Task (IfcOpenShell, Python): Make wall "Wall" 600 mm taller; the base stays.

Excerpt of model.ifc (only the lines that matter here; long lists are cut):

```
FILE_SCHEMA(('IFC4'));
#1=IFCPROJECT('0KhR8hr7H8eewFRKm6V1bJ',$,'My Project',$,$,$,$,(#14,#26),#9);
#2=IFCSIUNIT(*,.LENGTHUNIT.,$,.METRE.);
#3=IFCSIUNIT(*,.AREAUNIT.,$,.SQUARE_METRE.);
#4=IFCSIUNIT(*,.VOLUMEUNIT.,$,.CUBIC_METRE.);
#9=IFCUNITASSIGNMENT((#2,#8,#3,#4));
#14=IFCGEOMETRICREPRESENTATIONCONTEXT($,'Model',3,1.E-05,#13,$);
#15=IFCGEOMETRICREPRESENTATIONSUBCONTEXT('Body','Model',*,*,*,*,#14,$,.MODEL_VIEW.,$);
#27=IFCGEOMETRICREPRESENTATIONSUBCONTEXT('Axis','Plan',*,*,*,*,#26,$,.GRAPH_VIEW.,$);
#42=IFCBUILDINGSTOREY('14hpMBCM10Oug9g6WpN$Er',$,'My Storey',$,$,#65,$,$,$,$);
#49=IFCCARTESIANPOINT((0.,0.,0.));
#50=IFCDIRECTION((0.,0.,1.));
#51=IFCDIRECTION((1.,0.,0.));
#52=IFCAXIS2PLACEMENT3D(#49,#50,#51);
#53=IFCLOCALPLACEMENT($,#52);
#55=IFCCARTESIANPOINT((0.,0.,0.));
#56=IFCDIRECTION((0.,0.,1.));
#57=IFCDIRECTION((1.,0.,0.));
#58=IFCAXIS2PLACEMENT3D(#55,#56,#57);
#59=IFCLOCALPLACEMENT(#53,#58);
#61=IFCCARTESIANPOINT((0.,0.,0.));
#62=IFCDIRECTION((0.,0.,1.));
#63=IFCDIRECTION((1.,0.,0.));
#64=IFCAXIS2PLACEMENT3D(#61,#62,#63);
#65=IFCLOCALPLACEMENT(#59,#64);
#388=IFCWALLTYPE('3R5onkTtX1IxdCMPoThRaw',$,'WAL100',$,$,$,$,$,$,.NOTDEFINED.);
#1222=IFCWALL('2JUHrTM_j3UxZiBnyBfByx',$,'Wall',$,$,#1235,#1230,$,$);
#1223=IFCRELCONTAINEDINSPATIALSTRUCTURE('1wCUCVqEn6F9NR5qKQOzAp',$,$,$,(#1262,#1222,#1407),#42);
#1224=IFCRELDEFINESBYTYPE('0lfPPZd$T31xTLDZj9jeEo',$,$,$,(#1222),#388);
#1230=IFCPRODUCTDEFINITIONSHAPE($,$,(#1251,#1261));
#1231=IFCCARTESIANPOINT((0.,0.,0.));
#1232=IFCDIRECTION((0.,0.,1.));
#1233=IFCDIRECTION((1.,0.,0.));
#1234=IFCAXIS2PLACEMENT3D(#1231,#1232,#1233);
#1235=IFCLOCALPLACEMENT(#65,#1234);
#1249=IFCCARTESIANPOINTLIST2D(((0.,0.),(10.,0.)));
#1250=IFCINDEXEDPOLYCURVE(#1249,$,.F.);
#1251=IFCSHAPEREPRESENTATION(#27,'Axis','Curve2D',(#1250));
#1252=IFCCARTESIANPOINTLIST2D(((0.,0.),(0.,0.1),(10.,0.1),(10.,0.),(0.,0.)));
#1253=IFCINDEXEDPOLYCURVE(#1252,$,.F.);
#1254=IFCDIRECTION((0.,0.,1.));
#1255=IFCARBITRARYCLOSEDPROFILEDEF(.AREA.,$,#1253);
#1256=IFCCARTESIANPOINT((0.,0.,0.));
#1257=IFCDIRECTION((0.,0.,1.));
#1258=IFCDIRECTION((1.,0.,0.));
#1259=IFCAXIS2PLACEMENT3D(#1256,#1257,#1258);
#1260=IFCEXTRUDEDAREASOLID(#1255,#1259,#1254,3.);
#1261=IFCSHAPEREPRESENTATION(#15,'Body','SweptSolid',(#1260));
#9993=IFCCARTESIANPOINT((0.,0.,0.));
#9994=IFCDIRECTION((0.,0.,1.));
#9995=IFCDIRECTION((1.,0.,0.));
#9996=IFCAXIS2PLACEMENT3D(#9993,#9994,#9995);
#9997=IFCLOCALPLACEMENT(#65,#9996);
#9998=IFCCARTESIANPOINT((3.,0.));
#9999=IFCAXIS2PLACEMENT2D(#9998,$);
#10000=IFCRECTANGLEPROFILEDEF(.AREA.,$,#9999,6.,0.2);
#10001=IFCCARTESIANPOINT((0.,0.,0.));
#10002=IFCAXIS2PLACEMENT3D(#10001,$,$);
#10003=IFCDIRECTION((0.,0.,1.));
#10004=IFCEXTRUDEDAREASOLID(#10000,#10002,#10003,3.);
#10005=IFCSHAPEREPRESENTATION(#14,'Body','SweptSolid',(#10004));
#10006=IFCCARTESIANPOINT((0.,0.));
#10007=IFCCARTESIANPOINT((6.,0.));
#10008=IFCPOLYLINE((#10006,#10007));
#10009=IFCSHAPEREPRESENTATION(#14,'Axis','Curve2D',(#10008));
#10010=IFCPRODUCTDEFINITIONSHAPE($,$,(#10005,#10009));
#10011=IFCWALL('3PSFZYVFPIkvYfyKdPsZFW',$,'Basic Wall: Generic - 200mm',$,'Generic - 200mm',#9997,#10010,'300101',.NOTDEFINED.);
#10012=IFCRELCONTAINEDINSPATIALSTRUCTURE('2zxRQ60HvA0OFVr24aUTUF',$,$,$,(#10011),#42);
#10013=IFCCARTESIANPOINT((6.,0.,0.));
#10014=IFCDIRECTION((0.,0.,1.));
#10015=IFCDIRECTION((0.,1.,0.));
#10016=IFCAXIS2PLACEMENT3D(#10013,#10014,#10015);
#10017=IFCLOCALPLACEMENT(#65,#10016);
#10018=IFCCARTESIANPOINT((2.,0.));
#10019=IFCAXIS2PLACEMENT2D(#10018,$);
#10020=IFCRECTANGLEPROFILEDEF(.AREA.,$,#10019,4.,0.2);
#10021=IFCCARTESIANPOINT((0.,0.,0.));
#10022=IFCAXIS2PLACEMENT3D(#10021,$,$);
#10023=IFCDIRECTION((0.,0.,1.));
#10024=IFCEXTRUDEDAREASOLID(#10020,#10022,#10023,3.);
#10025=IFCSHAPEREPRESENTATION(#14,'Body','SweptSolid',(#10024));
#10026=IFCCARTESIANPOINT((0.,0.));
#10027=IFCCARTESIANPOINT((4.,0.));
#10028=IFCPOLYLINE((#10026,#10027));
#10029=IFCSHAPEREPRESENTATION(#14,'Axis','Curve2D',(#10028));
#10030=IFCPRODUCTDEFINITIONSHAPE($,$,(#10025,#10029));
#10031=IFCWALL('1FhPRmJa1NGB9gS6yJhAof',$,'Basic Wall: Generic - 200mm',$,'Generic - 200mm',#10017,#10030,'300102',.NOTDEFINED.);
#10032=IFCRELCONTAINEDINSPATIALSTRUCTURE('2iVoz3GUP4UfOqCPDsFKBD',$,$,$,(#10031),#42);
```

```python
import ifcopenshell
import ifcopenshell.geom
import ifcopenshell.util.representation
import ifcopenshell.util.shape

model = ifcopenshell.open("model.ifc")
settings = ifcopenshell.geom.settings()


def volume(element):
    """Net volume in cubic metres, openings subtracted."""
    shape = ifcopenshell.geom.create_shape(settings, element)
    return ifcopenshell.util.shape.get_volume(shape.geometry)


wall = model.by_guid("2JUHrTM_j3UxZiBnyBfByx")
before = volume(wall)

body = ifcopenshell.util.representation.get_representation(wall, "Model", "Body")
solid = body.Items[0]
old_height = solid.Depth
solid.Depth += 0.6
after = volume(wall)

print(f"height {old_height:g} -> {solid.Depth:g}, volume {before:.3f} -> {after:.3f} m3")

model.write("model_edited.ifc")
```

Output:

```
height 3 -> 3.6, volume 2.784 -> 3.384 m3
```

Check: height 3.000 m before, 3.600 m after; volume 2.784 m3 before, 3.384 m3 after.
